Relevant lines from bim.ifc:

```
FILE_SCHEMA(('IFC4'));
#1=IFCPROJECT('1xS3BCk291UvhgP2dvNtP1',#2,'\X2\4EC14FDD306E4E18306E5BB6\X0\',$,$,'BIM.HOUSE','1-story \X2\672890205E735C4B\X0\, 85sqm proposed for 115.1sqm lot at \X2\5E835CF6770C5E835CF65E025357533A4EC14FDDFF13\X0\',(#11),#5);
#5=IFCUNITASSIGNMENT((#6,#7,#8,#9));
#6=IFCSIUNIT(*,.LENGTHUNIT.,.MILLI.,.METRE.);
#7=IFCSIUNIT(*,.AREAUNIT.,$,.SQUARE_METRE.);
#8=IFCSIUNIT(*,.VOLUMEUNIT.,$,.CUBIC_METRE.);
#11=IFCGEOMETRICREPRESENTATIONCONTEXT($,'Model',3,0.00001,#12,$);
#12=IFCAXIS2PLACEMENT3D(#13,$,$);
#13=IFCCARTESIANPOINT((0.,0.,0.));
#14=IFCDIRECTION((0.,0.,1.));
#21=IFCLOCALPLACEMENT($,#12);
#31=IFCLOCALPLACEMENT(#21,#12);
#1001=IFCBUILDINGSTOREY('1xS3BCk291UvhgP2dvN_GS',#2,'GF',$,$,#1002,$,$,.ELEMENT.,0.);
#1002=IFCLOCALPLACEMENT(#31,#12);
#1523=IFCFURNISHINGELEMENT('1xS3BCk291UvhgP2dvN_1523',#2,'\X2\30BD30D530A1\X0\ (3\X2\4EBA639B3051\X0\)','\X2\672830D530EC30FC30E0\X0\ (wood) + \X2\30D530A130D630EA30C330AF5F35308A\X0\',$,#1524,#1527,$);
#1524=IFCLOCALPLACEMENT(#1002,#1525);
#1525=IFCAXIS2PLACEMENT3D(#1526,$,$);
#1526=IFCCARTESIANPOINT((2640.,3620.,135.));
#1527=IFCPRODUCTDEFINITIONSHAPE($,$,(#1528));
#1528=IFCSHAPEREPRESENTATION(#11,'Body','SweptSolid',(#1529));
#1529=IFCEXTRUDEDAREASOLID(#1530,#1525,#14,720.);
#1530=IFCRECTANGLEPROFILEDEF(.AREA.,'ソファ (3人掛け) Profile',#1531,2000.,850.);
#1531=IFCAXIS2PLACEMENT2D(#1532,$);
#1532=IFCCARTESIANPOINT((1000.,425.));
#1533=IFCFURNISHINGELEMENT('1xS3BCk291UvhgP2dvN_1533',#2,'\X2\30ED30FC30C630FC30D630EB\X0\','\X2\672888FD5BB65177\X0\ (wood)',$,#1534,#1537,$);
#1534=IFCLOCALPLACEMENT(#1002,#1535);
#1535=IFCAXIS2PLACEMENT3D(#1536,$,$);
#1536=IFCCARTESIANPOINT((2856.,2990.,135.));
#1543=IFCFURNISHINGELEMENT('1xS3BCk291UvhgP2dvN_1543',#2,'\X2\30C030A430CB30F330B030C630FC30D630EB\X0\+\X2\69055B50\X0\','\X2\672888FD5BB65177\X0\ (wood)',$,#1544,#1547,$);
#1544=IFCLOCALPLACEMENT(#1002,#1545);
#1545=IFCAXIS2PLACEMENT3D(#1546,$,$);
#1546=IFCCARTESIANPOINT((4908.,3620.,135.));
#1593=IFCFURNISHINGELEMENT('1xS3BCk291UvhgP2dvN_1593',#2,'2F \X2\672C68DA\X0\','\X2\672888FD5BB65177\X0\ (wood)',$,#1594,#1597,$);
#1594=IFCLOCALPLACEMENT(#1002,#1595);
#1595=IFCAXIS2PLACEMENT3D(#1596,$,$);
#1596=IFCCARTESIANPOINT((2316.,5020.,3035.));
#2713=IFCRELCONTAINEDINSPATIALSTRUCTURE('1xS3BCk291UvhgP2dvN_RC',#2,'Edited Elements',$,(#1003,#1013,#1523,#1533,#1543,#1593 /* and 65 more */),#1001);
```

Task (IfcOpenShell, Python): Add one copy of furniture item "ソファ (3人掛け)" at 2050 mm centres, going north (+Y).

```python
import numpy as np
import ifcopenshell
import ifcopenshell.api.geometry
import ifcopenshell.api.root
import ifcopenshell.util.element
import ifcopenshell.util.placement
import ifcopenshell.util.unit

model = ifcopenshell.open("bim.ifc")
unit_scale = ifcopenshell.util.unit.calculate_unit_scale(model)


def reuse_history(source, copy):
    """copy_class also copies each property set's owner history, people and application; keep the originals."""
    for rel in copy.IsDefinedBy:
        if rel.is_a("IfcRelDefinesByProperties") and (history := rel.RelatingPropertyDefinition.OwnerHistory):
            rel.RelatingPropertyDefinition.OwnerHistory = source.OwnerHistory
            ifcopenshell.util.element.remove_deep2(model, history)


source = model.by_guid("1xS3BCk291UvhgP2dvN_1523")
base = ifcopenshell.util.placement.get_local_placement(source.ObjectPlacement)
step = np.array([0.0, 1.0, 0.0]) * 2.05 / unit_scale

for i in range(1, 2):
    copy = ifcopenshell.api.root.copy_class(model, product=source)
    copy.Representation = ifcopenshell.util.element.copy_deep(
        model, source.Representation, exclude=["IfcGeometricRepresentationContext", "IfcRepresentationMap"]
    )
    reuse_history(source, copy)
    matrix = base.copy()
    matrix[:3, 3] += i * step
    print("added at", matrix[:3, 3].round(3) + 0.0)
    ifcopenshell.api.geometry.edit_object_placement(model, product=copy, matrix=matrix, is_si=False)

model.write("bim_rev.ifc")
```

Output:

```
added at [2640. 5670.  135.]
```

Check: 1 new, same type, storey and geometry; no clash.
